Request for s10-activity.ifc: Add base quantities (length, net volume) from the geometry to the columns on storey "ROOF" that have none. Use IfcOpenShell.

First a look at what the model holds.

```python
import ifcopenshell
import ifcopenshell.util.element
import ifcopenshell.util.unit

model = ifcopenshell.open("s10-activity.ifc")
print(model.schema)
for unit_type in ("LENGTHUNIT", "AREAUNIT", "VOLUMEUNIT"):
    print(unit_type, ifcopenshell.util.unit.calculate_unit_scale(model, unit_type))
storey = next(s for s in model.by_type("IfcBuildingStorey") if s.Name == "ROOF")
columns = [e for e in ifcopenshell.util.element.get_decomposition(storey) if e.is_a("IfcColumn")]
for e in sorted(columns, key=lambda e: e.id()):
    print(e.id(), e.is_a(), e.Name, list(ifcopenshell.util.element.get_psets(e, qtos_only=True)), sep=" | ")
```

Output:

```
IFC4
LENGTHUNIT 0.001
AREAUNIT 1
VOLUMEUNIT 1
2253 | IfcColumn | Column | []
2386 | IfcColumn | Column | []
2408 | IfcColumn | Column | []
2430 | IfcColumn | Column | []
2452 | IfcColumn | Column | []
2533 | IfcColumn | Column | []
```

```python
import ifcopenshell
import ifcopenshell.api.pset
import ifcopenshell.geom
import ifcopenshell.util.element
import ifcopenshell.util.shape
import ifcopenshell.util.unit

model = ifcopenshell.open("s10-activity.ifc")
unit_scale = ifcopenshell.util.unit.calculate_unit_scale(model)
volume_scale = ifcopenshell.util.unit.calculate_unit_scale(model, "VOLUMEUNIT")
settings = ifcopenshell.geom.settings()

storey = next(s for s in model.by_type("IfcBuildingStorey") if s.Name == "ROOF")
columns = [e for e in ifcopenshell.util.element.get_decomposition(storey) if e.is_a("IfcColumn")]

for e in sorted(columns, key=lambda e: e.id()):
    if ifcopenshell.util.element.get_psets(e, qtos_only=True, should_inherit=False):
        continue
    # Geometry comes back in metres, in the element's own axes.
    shape = ifcopenshell.geom.create_shape(settings, e)
    values = {
        "Length": ifcopenshell.util.shape.get_z(shape.geometry) / unit_scale,
        "NetVolume": ifcopenshell.util.shape.get_volume(shape.geometry) / volume_scale,
    }
    qto = ifcopenshell.api.pset.add_qto(model, product=e, name="Qto_ColumnBaseQuantities")
    ifcopenshell.api.pset.edit_qto(model, qto=qto, properties=values)
    print(e.id(), {k: round(v, 3) for k, v in values.items()})

model.write("s10-activity_rev.ifc")
```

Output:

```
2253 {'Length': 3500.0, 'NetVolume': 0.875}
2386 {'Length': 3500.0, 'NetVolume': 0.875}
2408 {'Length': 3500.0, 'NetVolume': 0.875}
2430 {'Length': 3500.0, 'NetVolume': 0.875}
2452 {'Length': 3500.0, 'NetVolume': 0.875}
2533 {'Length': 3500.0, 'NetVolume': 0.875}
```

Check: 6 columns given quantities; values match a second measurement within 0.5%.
